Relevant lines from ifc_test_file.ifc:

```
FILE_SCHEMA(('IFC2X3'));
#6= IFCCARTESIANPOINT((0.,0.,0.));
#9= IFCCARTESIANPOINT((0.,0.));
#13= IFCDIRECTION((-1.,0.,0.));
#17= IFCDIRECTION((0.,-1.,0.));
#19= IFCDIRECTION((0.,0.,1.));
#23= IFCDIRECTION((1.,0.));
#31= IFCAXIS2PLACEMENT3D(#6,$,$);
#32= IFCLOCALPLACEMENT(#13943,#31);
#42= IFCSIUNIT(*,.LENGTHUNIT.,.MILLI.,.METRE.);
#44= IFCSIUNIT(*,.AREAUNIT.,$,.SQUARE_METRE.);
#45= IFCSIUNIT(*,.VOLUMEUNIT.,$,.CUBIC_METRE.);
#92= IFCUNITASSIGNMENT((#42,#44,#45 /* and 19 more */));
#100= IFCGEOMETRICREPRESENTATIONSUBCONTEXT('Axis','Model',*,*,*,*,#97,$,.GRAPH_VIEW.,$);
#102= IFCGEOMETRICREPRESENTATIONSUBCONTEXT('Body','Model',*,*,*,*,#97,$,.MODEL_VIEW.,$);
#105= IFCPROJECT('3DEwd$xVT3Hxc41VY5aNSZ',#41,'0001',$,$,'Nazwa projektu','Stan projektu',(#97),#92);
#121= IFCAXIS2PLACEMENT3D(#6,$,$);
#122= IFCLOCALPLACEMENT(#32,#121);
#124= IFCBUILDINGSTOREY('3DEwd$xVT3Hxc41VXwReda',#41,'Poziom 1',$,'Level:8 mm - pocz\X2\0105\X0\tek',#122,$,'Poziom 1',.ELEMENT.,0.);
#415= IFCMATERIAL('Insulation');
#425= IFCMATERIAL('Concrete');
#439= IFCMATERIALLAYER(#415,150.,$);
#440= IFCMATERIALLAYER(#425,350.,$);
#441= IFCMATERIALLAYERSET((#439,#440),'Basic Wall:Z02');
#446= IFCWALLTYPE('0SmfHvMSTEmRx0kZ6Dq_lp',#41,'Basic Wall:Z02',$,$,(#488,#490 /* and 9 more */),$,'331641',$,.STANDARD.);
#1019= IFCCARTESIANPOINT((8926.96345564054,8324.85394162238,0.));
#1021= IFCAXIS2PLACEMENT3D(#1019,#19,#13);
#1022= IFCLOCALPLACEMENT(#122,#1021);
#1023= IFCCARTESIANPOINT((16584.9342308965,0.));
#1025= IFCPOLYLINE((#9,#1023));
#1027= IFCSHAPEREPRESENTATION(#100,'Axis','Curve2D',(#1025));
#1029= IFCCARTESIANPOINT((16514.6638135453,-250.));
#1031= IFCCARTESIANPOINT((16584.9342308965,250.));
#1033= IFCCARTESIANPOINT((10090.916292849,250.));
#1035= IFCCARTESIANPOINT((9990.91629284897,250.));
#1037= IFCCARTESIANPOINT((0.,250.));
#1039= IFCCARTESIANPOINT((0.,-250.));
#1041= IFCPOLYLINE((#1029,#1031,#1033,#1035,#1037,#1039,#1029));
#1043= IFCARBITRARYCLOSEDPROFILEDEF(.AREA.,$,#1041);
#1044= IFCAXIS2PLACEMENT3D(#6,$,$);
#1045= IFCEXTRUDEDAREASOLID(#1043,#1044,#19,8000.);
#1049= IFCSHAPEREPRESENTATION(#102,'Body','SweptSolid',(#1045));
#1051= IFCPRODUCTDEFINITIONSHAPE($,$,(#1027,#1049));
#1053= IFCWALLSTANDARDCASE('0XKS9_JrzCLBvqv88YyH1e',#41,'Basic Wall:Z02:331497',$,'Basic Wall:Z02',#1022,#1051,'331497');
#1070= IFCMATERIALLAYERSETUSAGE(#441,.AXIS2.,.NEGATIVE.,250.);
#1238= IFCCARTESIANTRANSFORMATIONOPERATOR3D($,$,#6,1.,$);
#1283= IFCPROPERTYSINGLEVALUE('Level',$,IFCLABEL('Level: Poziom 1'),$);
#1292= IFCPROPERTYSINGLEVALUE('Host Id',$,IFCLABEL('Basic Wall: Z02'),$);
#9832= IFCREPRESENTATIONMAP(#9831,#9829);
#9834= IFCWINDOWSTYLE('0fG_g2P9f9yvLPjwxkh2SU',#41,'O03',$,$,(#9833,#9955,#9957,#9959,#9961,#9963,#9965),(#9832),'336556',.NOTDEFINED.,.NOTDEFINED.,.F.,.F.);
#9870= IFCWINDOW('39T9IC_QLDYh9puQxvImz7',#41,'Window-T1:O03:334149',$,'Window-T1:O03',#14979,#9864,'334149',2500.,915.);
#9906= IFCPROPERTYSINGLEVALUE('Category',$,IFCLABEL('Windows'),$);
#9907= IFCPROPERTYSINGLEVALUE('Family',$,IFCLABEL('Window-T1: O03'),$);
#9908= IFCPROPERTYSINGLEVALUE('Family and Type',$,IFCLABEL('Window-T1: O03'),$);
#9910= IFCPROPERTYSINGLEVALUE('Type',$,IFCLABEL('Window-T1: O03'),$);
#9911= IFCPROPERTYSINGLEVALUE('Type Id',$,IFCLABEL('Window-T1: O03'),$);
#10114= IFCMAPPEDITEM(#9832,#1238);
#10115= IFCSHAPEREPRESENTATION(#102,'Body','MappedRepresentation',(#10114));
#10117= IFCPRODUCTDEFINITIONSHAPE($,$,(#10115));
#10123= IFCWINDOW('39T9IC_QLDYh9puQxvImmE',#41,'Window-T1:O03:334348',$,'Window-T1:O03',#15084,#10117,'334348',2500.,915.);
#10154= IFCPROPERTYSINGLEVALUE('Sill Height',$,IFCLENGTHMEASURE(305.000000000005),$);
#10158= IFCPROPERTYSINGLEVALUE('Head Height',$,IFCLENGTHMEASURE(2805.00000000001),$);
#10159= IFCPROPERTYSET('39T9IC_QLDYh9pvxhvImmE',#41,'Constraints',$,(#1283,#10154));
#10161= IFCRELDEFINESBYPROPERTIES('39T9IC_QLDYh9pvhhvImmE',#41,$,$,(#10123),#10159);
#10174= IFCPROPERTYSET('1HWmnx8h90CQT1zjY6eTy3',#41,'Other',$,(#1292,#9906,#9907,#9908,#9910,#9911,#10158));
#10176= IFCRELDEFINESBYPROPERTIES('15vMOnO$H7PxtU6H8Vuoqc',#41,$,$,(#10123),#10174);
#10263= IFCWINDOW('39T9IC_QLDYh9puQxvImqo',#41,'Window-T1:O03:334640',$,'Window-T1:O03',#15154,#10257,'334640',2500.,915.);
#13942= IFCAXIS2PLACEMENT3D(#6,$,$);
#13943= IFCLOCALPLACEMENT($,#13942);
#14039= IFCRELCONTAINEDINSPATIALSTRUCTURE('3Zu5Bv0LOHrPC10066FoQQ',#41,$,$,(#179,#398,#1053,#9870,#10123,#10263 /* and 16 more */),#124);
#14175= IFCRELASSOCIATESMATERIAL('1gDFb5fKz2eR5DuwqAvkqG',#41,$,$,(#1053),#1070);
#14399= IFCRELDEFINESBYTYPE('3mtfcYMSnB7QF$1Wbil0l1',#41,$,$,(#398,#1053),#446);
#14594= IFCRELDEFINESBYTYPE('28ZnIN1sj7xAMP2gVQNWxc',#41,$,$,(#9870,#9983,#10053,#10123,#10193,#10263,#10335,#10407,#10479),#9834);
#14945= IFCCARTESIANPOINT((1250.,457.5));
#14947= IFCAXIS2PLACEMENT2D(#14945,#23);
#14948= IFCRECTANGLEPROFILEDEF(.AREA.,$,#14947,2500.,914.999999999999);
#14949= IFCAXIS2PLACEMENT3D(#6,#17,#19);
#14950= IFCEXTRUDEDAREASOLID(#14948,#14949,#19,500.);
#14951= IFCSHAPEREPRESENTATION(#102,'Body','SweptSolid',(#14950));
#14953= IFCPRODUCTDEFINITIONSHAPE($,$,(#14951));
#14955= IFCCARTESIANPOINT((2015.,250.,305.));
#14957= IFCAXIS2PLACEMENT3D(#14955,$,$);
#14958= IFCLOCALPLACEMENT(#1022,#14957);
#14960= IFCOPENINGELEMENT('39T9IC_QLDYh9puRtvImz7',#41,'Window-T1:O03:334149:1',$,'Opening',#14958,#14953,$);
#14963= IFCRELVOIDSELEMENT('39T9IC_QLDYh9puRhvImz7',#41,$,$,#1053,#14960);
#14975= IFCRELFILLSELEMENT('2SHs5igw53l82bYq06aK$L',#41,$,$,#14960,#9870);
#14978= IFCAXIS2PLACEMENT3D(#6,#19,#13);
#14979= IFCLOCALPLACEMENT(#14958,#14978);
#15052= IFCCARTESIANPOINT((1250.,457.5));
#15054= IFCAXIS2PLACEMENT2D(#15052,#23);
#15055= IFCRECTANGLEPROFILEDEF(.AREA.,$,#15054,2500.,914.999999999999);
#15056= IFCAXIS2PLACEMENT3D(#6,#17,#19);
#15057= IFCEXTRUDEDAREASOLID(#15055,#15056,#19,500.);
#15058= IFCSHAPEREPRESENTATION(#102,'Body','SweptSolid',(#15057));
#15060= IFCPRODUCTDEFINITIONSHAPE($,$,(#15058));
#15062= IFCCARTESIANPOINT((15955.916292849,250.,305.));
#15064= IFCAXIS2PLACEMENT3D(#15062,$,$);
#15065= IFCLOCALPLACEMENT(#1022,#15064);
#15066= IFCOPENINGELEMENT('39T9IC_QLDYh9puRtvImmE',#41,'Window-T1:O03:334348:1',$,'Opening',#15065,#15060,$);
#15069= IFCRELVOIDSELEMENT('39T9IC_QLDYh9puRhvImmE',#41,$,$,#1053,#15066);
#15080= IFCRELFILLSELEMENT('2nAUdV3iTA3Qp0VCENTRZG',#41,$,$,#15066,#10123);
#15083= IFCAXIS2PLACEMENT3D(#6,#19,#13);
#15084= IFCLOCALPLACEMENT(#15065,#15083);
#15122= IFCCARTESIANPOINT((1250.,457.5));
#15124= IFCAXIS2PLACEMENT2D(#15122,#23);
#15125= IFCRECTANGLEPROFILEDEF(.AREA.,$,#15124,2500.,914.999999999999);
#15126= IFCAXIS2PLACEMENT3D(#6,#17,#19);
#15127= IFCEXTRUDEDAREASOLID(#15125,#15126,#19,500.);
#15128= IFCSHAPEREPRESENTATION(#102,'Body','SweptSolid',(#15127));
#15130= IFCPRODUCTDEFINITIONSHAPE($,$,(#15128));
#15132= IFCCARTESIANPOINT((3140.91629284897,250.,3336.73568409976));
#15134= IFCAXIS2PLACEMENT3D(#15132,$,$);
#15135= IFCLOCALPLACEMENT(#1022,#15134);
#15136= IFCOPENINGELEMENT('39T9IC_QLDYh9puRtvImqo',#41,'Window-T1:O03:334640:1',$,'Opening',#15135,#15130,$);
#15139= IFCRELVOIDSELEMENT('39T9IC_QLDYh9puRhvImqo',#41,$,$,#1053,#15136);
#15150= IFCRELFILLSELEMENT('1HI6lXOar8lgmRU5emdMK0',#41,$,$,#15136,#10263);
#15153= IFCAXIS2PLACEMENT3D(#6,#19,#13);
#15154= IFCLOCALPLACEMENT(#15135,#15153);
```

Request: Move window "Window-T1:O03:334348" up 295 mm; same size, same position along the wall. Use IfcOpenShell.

```python
import numpy as np
import ifcopenshell
import ifcopenshell.api.geometry
import ifcopenshell.api.pset
import ifcopenshell.util.element
import ifcopenshell.util.placement
import ifcopenshell.util.unit

model = ifcopenshell.open("ifc_test_file.ifc")
unit_scale = ifcopenshell.util.unit.calculate_unit_scale(model)

window = model.by_guid("39T9IC_QLDYh9puQxvImmE")
opening = window.FillsVoids[0].RelatingOpeningElement
dz = 0.295 / unit_scale

shift = np.array([0.0, 0.0, dz])
# The window is placed relative to its opening, so it follows when the opening moves.
matrix = ifcopenshell.util.placement.get_local_placement(opening.ObjectPlacement)
matrix[:3, 3] += shift
ifcopenshell.api.geometry.edit_object_placement(
    model, product=opening, matrix=matrix, is_si=False, should_transform_children=True
)

# Keep the stored heights in step.
pset = model.by_id(ifcopenshell.util.element.get_pset(window, "Constraints", should_inherit=False)["id"])
ifcopenshell.api.pset.edit_pset(model, pset=pset, properties={
    "Sill Height": model.create_entity("IfcLengthMeasure", ifcopenshell.util.element.get_pset(window, "Constraints", "Sill Height") + dz),
})
pset = model.by_id(ifcopenshell.util.element.get_pset(window, "Other", should_inherit=False)["id"])
ifcopenshell.api.pset.edit_pset(model, pset=pset, properties={
    "Head Height": model.create_entity("IfcLengthMeasure", ifcopenshell.util.element.get_pset(window, "Other", "Head Height") + dz),
})

print(f"moved by {dz * unit_scale:+.3f} m")

model.write("ifc_test_file_v2.ifc")
```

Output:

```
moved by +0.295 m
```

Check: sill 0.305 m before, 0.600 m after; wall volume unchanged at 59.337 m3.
